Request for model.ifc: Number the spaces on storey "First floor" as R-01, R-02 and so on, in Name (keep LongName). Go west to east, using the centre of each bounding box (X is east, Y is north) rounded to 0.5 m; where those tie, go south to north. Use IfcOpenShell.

First a look at what the model holds.

```python
import ifcopenshell
import ifcopenshell.util.element
import ifcopenshell.util.placement

model = ifcopenshell.open("model.ifc")
print(model.schema)
storey = next(s for s in model.by_type("IfcBuildingStorey") if s.Name == "First floor")
spaces = [e for e in ifcopenshell.util.element.get_decomposition(storey) if e.is_a("IfcSpace")]
for e in sorted(spaces, key=lambda e: e.id()):
    origin = ifcopenshell.util.placement.get_local_placement(e.ObjectPlacement)[:3, 3]
    print(e.id(), e.Name, e.LongName, origin.round(2) + 0.0, sep=" | ")
```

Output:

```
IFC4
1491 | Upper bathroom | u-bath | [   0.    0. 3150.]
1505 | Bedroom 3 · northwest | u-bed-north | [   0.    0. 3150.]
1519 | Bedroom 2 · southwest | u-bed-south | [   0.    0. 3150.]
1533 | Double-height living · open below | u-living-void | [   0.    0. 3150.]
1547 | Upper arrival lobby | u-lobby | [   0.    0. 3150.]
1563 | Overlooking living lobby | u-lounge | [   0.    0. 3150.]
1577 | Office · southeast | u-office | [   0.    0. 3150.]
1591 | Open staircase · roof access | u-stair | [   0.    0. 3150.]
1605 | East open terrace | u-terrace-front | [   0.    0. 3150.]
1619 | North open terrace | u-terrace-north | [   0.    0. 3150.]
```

```python
import ifcopenshell
import ifcopenshell.geom
import ifcopenshell.util.element
import ifcopenshell.util.shape

model = ifcopenshell.open("model.ifc")
settings = ifcopenshell.geom.settings()
settings.set("use-world-coords", True)


def centre(element):
    shape = ifcopenshell.geom.create_shape(settings, element)
    return ifcopenshell.util.shape.get_bbox_centroid(shape.geometry)


storey = next(s for s in model.by_type("IfcBuildingStorey") if s.Name == "First floor")
spaces = [e for e in ifcopenshell.util.element.get_decomposition(storey) if e.is_a("IfcSpace")]

# Insertion points can sit at a corner or the storey origin, so sort by the geometry (in metres).
centres = {e: centre(e) for e in spaces}
spaces.sort(key=lambda e: (round(centres[e][0] / 0.5), centres[e][1]))

for i, e in enumerate(spaces, start=1):
    number = f"R-{i:02d}"
    e.Name = number
    print(e.id(), number)

model.write("model_rev.ifc")
```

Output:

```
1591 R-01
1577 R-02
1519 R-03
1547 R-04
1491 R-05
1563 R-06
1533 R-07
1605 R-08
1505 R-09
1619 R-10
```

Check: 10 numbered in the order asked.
